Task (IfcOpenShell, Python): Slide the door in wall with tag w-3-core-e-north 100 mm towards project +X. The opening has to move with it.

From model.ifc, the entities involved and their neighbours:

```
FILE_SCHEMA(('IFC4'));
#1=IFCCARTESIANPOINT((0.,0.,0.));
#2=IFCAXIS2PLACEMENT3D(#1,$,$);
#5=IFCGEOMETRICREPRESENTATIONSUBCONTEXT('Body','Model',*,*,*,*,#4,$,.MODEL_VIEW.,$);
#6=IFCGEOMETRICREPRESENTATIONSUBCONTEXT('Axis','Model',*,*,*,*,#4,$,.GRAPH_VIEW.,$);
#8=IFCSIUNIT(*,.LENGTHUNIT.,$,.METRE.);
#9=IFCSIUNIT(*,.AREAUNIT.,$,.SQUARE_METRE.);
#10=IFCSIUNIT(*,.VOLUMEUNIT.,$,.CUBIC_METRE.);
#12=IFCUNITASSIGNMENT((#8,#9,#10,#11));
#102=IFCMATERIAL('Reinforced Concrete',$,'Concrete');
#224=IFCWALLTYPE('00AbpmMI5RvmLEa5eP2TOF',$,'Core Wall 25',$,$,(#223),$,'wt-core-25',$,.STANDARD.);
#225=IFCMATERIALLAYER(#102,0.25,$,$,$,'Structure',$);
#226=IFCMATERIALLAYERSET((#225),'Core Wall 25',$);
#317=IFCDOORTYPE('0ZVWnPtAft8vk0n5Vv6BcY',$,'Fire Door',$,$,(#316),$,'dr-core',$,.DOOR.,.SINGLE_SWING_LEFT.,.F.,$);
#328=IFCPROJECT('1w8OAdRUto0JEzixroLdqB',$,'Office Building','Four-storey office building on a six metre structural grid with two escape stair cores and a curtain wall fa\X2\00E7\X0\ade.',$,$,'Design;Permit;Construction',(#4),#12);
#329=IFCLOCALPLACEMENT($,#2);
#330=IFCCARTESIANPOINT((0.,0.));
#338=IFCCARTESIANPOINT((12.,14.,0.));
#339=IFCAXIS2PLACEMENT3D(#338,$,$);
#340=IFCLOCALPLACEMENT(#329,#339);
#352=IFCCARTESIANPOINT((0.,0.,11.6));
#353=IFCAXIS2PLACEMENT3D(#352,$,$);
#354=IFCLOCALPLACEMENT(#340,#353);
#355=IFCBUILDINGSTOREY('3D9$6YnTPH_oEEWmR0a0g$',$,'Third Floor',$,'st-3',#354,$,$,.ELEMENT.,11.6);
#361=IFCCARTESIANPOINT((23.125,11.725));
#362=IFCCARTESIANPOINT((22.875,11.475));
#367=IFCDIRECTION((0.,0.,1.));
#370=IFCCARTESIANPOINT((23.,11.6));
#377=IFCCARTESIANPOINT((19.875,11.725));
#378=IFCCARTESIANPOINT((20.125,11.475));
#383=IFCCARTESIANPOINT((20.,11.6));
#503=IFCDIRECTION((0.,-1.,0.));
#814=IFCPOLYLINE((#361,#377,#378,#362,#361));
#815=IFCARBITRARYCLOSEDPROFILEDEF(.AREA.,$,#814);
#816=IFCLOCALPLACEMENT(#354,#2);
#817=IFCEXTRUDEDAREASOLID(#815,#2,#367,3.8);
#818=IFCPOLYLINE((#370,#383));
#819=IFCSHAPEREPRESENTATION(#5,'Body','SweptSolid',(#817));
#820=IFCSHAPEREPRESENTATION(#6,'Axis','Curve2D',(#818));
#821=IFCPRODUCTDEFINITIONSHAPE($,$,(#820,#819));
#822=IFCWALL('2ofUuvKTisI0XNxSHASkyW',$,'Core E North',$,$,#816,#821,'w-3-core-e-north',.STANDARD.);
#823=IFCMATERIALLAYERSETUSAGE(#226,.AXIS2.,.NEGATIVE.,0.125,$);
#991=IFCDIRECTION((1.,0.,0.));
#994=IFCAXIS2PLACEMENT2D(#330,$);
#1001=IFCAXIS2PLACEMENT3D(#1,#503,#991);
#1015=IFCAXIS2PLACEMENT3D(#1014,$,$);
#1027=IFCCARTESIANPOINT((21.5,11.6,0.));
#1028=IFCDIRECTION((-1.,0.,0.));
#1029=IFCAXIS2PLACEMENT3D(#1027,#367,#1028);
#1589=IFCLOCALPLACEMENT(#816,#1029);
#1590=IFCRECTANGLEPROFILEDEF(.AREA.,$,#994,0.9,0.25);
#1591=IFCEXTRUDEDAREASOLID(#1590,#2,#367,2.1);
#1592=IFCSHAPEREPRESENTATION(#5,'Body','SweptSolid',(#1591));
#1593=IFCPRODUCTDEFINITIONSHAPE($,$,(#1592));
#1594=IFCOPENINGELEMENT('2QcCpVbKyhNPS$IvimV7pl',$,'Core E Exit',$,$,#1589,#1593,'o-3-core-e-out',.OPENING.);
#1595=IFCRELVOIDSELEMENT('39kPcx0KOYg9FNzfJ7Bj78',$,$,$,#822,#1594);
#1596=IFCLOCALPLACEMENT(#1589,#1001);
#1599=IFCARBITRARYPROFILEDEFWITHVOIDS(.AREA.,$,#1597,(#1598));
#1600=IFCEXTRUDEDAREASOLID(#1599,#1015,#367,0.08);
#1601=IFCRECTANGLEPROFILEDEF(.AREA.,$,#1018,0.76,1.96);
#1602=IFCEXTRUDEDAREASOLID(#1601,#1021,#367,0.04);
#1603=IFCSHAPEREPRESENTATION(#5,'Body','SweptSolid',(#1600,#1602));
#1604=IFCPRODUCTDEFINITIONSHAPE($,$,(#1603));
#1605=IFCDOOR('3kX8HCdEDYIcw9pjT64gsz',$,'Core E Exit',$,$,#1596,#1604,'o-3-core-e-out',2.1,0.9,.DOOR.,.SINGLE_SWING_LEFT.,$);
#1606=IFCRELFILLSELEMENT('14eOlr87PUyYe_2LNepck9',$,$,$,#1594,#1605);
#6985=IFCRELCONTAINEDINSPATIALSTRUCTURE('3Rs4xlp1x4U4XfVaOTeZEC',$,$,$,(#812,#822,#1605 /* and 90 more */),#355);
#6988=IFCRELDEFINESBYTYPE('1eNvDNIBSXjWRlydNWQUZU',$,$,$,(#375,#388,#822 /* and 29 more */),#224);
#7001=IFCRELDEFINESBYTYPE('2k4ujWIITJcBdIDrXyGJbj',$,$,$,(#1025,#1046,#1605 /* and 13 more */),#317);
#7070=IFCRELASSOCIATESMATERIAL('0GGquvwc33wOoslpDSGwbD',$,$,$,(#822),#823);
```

```python
import ifcopenshell
import ifcopenshell.api.geometry
import ifcopenshell.util.placement
import ifcopenshell.util.unit

model = ifcopenshell.open("model.ifc")
unit_scale = ifcopenshell.util.unit.calculate_unit_scale(model)

door = model.by_guid("3kX8HCdEDYIcw9pjT64gsz")
opening = door.FillsVoids[0].RelatingOpeningElement
wall = opening.VoidsElements[0].RelatingBuildingElement

wall_matrix = ifcopenshell.util.placement.get_local_placement(wall.ObjectPlacement)
shift = wall_matrix[:3, 0] * 0.1 / unit_scale
before = ifcopenshell.util.placement.get_local_placement(door.ObjectPlacement)[:3, 3].copy()

# The door is placed relative to its opening, so it follows when the opening moves.
matrix = ifcopenshell.util.placement.get_local_placement(opening.ObjectPlacement)
matrix[:3, 3] += shift
ifcopenshell.api.geometry.edit_object_placement(
    model, product=opening, matrix=matrix, is_si=False, should_transform_children=True
)

after = ifcopenshell.util.placement.get_local_placement(door.ObjectPlacement)[:3, 3]
print("door moved by", (after - before).round(3) + 0.0)

model.write("model-out.ifc")
```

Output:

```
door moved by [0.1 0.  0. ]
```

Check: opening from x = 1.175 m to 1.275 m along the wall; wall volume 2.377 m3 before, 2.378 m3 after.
